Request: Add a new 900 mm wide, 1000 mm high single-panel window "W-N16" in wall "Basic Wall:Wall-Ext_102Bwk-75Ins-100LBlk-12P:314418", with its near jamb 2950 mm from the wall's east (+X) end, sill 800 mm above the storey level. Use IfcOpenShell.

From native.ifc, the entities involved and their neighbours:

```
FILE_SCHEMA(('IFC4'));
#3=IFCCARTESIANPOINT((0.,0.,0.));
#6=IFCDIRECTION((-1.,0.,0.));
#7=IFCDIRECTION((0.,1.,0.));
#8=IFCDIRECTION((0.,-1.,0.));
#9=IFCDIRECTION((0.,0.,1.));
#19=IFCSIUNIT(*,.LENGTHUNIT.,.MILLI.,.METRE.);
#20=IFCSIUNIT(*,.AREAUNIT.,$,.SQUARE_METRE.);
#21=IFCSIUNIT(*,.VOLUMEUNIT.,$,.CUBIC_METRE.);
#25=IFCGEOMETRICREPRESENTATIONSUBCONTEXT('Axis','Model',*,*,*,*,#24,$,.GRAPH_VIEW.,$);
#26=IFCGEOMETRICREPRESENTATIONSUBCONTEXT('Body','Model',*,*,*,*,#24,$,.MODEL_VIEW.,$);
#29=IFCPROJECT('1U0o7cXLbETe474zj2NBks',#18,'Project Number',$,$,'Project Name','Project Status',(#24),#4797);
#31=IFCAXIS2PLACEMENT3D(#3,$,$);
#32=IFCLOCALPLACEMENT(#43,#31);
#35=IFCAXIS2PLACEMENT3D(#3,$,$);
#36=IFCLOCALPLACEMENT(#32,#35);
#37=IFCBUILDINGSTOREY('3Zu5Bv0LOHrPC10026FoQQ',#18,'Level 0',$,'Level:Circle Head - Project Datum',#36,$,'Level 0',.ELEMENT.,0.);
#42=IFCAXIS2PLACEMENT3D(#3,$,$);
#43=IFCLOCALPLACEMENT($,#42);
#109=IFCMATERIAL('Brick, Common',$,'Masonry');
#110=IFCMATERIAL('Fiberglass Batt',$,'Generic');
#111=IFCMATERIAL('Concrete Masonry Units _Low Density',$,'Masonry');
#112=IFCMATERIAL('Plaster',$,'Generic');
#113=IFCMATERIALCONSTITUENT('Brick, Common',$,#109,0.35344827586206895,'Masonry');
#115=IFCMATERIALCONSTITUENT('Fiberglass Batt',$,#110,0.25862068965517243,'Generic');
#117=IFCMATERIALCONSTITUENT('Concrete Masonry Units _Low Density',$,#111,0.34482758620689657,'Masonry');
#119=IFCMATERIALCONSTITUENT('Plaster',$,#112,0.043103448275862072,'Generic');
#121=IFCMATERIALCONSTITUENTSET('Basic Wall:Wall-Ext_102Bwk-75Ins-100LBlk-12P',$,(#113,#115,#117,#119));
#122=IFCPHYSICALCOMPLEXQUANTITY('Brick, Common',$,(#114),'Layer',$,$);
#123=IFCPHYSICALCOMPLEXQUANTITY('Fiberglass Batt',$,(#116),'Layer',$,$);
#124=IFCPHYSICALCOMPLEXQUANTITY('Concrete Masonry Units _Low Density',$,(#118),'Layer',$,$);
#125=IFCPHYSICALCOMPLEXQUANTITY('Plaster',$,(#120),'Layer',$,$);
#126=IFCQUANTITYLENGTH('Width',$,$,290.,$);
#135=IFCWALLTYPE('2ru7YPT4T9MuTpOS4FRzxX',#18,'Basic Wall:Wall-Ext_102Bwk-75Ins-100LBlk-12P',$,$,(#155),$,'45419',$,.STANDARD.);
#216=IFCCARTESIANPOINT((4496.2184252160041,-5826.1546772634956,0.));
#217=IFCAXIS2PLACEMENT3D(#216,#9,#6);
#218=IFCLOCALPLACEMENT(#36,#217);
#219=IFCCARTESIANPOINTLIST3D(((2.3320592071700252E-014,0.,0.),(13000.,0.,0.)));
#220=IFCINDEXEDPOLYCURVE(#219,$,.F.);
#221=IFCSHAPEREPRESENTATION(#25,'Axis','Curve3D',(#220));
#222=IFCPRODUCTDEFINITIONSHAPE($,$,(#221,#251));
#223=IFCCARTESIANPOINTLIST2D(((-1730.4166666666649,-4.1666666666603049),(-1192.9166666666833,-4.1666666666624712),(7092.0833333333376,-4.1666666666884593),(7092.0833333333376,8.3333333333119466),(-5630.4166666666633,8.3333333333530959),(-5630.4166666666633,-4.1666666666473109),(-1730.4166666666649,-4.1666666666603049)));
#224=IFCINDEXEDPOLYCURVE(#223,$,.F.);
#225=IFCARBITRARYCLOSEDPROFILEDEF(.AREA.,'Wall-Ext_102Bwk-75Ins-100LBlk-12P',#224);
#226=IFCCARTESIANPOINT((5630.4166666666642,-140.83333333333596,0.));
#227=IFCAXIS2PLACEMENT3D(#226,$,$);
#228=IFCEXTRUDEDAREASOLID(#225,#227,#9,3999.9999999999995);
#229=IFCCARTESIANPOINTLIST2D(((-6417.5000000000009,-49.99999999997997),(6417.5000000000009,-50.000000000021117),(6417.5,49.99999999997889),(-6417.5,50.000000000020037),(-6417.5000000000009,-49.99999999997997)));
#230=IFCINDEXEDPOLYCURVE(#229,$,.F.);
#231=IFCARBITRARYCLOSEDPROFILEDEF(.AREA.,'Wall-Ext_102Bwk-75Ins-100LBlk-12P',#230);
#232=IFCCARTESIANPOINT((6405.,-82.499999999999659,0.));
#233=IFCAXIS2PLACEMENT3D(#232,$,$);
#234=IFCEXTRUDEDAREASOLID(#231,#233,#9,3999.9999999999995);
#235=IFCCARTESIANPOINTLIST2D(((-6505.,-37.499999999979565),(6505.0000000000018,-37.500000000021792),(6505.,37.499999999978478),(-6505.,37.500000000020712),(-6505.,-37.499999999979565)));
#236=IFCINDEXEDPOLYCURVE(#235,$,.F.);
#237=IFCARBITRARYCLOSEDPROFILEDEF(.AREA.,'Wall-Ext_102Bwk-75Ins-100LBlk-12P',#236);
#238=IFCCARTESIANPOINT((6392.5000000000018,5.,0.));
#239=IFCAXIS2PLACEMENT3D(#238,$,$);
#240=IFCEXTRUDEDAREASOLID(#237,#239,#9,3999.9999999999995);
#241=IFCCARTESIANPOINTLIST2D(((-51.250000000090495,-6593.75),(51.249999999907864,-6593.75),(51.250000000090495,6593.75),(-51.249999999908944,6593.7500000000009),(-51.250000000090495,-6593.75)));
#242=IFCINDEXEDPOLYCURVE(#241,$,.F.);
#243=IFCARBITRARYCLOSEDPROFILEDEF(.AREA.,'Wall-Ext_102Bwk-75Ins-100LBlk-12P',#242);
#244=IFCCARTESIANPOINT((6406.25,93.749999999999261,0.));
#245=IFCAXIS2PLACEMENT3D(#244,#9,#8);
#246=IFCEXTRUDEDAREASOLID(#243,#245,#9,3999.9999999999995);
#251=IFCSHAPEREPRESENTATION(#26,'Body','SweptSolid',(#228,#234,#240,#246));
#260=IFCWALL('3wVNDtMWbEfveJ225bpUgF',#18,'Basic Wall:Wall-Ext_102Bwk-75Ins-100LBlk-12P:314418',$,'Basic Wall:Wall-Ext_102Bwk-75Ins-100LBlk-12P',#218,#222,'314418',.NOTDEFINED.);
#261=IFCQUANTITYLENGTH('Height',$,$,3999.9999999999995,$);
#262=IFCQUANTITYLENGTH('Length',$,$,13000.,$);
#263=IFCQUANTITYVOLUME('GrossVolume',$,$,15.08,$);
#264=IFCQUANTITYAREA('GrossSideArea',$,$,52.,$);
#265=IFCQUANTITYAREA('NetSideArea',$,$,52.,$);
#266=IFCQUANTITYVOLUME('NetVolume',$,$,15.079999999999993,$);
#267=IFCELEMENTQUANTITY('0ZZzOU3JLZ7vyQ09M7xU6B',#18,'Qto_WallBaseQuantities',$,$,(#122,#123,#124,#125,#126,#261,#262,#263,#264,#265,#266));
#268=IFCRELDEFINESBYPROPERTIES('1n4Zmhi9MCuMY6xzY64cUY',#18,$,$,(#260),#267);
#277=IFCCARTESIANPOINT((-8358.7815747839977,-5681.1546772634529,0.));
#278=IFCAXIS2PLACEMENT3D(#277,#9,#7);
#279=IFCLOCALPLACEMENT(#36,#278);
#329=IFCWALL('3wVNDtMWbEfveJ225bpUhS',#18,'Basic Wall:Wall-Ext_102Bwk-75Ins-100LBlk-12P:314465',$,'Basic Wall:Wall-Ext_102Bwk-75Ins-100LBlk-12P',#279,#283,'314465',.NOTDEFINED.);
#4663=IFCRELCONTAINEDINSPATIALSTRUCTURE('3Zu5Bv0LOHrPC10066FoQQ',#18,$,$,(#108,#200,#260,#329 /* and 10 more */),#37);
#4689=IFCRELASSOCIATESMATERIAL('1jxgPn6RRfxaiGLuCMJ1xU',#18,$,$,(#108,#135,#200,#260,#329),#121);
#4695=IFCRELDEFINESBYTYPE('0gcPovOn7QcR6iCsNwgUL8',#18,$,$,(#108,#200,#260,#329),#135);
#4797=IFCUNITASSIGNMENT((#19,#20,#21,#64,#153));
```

```python
import numpy as np
import ifcopenshell
import ifcopenshell.api.feature
import ifcopenshell.api.geometry
import ifcopenshell.api.pset
import ifcopenshell.api.root
import ifcopenshell.api.spatial
import ifcopenshell.geom
import ifcopenshell.util.element
import ifcopenshell.util.placement
import ifcopenshell.util.representation
import ifcopenshell.util.shape
import ifcopenshell.util.unit

model = ifcopenshell.open("native.ifc")
unit_scale = ifcopenshell.util.unit.calculate_unit_scale(model)
area_scale = ifcopenshell.util.unit.calculate_unit_scale(model, "AREAUNIT")
volume_scale = ifcopenshell.util.unit.calculate_unit_scale(model, "VOLUMEUNIT")
settings = ifcopenshell.geom.settings()


def volume(element):
    """Net volume in cubic metres, openings subtracted."""
    shape = ifcopenshell.geom.create_shape(settings, element)
    return ifcopenshell.util.shape.get_volume(shape.geometry)


wall = model.by_guid("3wVNDtMWbEfveJ225bpUgF")
storey = ifcopenshell.util.element.get_container(wall, ifc_class="IfcBuildingStorey")
context = ifcopenshell.util.representation.get_context(model, "Model", "Body", "MODEL_VIEW")
before = volume(wall)

width, height, from_end, sill = 0.9, 1, 2.95, 0.8  # metres

# The wall runs along its own X axis, and the end named is its -X end.
wall_shape = ifcopenshell.geom.create_shape(settings, wall)
x, y, z = ifcopenshell.util.shape.get_vertices(wall_shape.geometry).T
start = x.min() + from_end
face, thickness = float(y.min()), float(y.max() - y.min())
wall_matrix = ifcopenshell.util.placement.get_local_placement(wall.ObjectPlacement)
level = ifcopenshell.util.placement.get_local_placement(storey.ObjectPlacement)[2, 3]


def in_wall(x, y):
    """Placement at x, y metres in the wall's axes, at sill height."""
    matrix = wall_matrix.copy()
    matrix[:, 3] = wall_matrix @ np.array([x / unit_scale, y / unit_scale, 0.0, 1.0])
    matrix[2, 3] = level + sill / unit_scale
    return matrix


# Opening: a box that overshoots both wall faces by 50 mm.
opening = ifcopenshell.api.root.create_entity(model, ifc_class="IfcOpeningElement", predefined_type="OPENING")
box = ifcopenshell.api.geometry.add_wall_representation(
    model, context=context, length=width, height=height, thickness=thickness + 0.1
)
ifcopenshell.api.geometry.assign_representation(model, product=opening, representation=box)
ifcopenshell.api.geometry.edit_object_placement(model, product=opening, matrix=in_wall(start, face - 0.05), is_si=False)
ifcopenshell.api.feature.add_feature(model, feature=opening, element=wall)

window = ifcopenshell.api.root.create_entity(model, ifc_class="IfcWindow", name="W-N16", predefined_type="WINDOW")
window.OverallWidth, window.OverallHeight = width / unit_scale, height / unit_scale
window.PartitioningType = "SINGLE_PANEL"
body = ifcopenshell.api.geometry.add_window_representation(
    model,
    context=context,
    overall_width=window.OverallWidth,
    overall_height=window.OverallHeight,
    partition_type="SINGLE_PANEL",
)
ifcopenshell.api.geometry.assign_representation(model, product=window, representation=body)
ifcopenshell.api.spatial.assign_container(model, products=[window], relating_structure=storey)
ifcopenshell.api.feature.add_filling(model, opening=opening, element=window)

# Centre the window in the wall's thickness.
ifcopenshell.api.geometry.edit_object_placement(model, product=window, matrix=in_wall(start, face), is_si=False)
window_shape = ifcopenshell.geom.create_shape(settings, window)
depth = ifcopenshell.util.shape.get_vertices(window_shape.geometry)[:, 1]
offset = face + thickness / 2 - (depth.min() + depth.max()) / 2
ifcopenshell.api.geometry.edit_object_placement(model, product=window, matrix=in_wall(start, offset), is_si=False)

after = volume(wall)

# Update the wall's stored quantities.
qto = model.by_id(ifcopenshell.util.element.get_pset(wall, "Qto_WallBaseQuantities", should_inherit=False)["id"])
ifcopenshell.api.pset.edit_qto(model, qto=qto, properties={
    "NetSideArea": after / thickness / area_scale,
    "NetVolume": after / volume_scale,
})

print(f"wall volume {before:.3f} -> {after:.3f} m3")

model.write("native_updated.ifc")
```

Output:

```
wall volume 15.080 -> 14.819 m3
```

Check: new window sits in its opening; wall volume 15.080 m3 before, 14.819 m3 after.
